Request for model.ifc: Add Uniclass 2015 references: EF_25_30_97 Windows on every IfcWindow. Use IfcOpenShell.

First a look at what the model holds.

```python
import ifcopenshell

model = ifcopenshell.open("model.ifc")
print(model.schema)
print("classifications:", [c.Name for c in model.by_type("IfcClassification")])
for ifc_class in ("IfcDoor", "IfcRoof", "IfcStair", "IfcWall", "IfcWindow"):
    print(ifc_class, len(model.by_type(ifc_class)))
```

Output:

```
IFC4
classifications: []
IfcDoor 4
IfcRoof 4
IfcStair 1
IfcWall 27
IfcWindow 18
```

```python
import ifcopenshell
import ifcopenshell.api.classification

model = ifcopenshell.open("model.ifc")

system = ifcopenshell.api.classification.add_classification(model, classification="Uniclass 2015")

codes = {
    "IfcWindow": ("EF_25_30_97", "Windows"),
}
for ifc_class, (code, name) in codes.items():
    products = model.by_type(ifc_class)
    ifcopenshell.api.classification.add_reference(
        model, products=products, classification=system, identification=code, name=name
    )
    print(code, len(products))

model.write("model_edited.ifc")
```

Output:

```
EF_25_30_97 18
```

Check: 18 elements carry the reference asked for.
